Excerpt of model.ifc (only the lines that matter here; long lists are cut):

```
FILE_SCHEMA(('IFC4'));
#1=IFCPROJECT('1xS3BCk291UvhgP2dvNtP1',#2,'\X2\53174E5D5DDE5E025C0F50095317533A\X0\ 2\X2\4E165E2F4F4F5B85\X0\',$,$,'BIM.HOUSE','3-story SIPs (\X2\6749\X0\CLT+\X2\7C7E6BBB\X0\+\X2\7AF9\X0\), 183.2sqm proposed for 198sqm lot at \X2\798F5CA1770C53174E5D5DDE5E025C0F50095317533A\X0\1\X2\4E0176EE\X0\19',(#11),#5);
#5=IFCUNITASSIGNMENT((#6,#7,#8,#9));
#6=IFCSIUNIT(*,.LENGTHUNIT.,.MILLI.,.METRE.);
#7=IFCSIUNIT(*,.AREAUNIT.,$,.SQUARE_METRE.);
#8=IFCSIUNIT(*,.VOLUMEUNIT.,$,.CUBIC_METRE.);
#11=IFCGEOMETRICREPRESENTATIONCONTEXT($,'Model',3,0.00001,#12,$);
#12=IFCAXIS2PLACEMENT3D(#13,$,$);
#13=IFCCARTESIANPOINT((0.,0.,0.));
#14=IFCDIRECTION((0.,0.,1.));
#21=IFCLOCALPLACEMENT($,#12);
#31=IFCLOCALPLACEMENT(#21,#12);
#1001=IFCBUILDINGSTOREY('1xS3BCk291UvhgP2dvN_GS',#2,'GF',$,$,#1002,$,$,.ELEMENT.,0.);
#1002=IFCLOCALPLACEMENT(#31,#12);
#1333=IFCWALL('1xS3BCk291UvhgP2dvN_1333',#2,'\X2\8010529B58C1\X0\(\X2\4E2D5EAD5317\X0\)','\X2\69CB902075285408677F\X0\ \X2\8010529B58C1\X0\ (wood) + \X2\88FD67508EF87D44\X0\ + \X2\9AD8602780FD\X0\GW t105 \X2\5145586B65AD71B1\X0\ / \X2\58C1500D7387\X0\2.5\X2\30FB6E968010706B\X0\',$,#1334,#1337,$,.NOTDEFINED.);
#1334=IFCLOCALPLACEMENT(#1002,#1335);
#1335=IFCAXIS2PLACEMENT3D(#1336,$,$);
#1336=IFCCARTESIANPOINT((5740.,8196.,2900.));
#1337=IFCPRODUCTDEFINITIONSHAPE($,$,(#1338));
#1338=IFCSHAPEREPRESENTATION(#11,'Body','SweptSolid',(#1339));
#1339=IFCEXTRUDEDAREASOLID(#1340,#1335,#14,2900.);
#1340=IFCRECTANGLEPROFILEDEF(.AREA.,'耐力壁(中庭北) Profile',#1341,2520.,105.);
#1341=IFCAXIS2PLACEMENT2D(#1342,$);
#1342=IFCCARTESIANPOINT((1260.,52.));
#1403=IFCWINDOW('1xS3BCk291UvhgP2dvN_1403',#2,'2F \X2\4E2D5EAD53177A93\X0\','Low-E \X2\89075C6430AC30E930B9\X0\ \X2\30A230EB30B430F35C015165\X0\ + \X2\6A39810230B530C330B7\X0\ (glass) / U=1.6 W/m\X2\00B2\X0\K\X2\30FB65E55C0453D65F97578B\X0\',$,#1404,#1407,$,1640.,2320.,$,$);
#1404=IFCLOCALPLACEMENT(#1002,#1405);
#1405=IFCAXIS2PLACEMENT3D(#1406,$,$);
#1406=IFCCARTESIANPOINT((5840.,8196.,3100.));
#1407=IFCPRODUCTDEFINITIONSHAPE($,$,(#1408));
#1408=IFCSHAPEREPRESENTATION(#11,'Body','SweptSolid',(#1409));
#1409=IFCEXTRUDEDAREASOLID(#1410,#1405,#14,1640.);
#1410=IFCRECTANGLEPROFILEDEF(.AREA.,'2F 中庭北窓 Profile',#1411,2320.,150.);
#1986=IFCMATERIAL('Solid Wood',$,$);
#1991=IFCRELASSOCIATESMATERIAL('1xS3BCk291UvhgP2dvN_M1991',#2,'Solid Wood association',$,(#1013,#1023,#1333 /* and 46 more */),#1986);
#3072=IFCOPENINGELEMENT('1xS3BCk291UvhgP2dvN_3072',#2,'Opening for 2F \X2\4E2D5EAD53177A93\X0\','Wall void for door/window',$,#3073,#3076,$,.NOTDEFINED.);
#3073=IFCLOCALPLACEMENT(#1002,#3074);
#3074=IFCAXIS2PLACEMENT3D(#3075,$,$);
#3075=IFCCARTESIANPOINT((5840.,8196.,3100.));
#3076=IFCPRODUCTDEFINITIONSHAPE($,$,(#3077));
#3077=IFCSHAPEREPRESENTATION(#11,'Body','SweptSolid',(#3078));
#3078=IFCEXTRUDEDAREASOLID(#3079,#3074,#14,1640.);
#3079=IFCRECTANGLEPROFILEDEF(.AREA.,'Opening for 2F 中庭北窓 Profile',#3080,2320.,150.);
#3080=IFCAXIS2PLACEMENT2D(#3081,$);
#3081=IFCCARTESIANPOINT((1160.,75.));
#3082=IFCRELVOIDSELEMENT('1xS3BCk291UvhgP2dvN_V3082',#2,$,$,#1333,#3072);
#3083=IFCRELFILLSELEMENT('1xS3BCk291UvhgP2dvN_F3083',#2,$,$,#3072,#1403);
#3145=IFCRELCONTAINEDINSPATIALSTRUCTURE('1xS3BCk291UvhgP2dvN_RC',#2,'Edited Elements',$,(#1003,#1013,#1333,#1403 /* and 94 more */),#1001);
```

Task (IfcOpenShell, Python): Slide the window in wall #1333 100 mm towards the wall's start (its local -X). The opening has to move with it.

```python
import ifcopenshell
import ifcopenshell.api.geometry
import ifcopenshell.util.placement

model = ifcopenshell.open("model.ifc")

window = model.by_guid("1xS3BCk291UvhgP2dvN_1403")
opening = window.FillsVoids[0].RelatingOpeningElement
wall = opening.VoidsElements[0].RelatingBuildingElement

wall_matrix = ifcopenshell.util.placement.get_local_placement(wall.ObjectPlacement)
shift = wall_matrix[:3, 0] * -100.0
before = ifcopenshell.util.placement.get_local_placement(window.ObjectPlacement)[:3, 3].copy()

# The window is not placed relative to its opening, so move both.
for product in (opening, window):
    matrix = ifcopenshell.util.placement.get_local_placement(product.ObjectPlacement)
    matrix[:3, 3] += shift
    ifcopenshell.api.geometry.edit_object_placement(model, product=product, matrix=matrix, is_si=False)

after = ifcopenshell.util.placement.get_local_placement(window.ObjectPlacement)[:3, 3]
print("window moved by", (after - before).round(3) + 0.0)

model.write("model_updated.ifc")
```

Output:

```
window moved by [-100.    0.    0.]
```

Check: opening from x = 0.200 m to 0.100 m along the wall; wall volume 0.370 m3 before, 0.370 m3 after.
